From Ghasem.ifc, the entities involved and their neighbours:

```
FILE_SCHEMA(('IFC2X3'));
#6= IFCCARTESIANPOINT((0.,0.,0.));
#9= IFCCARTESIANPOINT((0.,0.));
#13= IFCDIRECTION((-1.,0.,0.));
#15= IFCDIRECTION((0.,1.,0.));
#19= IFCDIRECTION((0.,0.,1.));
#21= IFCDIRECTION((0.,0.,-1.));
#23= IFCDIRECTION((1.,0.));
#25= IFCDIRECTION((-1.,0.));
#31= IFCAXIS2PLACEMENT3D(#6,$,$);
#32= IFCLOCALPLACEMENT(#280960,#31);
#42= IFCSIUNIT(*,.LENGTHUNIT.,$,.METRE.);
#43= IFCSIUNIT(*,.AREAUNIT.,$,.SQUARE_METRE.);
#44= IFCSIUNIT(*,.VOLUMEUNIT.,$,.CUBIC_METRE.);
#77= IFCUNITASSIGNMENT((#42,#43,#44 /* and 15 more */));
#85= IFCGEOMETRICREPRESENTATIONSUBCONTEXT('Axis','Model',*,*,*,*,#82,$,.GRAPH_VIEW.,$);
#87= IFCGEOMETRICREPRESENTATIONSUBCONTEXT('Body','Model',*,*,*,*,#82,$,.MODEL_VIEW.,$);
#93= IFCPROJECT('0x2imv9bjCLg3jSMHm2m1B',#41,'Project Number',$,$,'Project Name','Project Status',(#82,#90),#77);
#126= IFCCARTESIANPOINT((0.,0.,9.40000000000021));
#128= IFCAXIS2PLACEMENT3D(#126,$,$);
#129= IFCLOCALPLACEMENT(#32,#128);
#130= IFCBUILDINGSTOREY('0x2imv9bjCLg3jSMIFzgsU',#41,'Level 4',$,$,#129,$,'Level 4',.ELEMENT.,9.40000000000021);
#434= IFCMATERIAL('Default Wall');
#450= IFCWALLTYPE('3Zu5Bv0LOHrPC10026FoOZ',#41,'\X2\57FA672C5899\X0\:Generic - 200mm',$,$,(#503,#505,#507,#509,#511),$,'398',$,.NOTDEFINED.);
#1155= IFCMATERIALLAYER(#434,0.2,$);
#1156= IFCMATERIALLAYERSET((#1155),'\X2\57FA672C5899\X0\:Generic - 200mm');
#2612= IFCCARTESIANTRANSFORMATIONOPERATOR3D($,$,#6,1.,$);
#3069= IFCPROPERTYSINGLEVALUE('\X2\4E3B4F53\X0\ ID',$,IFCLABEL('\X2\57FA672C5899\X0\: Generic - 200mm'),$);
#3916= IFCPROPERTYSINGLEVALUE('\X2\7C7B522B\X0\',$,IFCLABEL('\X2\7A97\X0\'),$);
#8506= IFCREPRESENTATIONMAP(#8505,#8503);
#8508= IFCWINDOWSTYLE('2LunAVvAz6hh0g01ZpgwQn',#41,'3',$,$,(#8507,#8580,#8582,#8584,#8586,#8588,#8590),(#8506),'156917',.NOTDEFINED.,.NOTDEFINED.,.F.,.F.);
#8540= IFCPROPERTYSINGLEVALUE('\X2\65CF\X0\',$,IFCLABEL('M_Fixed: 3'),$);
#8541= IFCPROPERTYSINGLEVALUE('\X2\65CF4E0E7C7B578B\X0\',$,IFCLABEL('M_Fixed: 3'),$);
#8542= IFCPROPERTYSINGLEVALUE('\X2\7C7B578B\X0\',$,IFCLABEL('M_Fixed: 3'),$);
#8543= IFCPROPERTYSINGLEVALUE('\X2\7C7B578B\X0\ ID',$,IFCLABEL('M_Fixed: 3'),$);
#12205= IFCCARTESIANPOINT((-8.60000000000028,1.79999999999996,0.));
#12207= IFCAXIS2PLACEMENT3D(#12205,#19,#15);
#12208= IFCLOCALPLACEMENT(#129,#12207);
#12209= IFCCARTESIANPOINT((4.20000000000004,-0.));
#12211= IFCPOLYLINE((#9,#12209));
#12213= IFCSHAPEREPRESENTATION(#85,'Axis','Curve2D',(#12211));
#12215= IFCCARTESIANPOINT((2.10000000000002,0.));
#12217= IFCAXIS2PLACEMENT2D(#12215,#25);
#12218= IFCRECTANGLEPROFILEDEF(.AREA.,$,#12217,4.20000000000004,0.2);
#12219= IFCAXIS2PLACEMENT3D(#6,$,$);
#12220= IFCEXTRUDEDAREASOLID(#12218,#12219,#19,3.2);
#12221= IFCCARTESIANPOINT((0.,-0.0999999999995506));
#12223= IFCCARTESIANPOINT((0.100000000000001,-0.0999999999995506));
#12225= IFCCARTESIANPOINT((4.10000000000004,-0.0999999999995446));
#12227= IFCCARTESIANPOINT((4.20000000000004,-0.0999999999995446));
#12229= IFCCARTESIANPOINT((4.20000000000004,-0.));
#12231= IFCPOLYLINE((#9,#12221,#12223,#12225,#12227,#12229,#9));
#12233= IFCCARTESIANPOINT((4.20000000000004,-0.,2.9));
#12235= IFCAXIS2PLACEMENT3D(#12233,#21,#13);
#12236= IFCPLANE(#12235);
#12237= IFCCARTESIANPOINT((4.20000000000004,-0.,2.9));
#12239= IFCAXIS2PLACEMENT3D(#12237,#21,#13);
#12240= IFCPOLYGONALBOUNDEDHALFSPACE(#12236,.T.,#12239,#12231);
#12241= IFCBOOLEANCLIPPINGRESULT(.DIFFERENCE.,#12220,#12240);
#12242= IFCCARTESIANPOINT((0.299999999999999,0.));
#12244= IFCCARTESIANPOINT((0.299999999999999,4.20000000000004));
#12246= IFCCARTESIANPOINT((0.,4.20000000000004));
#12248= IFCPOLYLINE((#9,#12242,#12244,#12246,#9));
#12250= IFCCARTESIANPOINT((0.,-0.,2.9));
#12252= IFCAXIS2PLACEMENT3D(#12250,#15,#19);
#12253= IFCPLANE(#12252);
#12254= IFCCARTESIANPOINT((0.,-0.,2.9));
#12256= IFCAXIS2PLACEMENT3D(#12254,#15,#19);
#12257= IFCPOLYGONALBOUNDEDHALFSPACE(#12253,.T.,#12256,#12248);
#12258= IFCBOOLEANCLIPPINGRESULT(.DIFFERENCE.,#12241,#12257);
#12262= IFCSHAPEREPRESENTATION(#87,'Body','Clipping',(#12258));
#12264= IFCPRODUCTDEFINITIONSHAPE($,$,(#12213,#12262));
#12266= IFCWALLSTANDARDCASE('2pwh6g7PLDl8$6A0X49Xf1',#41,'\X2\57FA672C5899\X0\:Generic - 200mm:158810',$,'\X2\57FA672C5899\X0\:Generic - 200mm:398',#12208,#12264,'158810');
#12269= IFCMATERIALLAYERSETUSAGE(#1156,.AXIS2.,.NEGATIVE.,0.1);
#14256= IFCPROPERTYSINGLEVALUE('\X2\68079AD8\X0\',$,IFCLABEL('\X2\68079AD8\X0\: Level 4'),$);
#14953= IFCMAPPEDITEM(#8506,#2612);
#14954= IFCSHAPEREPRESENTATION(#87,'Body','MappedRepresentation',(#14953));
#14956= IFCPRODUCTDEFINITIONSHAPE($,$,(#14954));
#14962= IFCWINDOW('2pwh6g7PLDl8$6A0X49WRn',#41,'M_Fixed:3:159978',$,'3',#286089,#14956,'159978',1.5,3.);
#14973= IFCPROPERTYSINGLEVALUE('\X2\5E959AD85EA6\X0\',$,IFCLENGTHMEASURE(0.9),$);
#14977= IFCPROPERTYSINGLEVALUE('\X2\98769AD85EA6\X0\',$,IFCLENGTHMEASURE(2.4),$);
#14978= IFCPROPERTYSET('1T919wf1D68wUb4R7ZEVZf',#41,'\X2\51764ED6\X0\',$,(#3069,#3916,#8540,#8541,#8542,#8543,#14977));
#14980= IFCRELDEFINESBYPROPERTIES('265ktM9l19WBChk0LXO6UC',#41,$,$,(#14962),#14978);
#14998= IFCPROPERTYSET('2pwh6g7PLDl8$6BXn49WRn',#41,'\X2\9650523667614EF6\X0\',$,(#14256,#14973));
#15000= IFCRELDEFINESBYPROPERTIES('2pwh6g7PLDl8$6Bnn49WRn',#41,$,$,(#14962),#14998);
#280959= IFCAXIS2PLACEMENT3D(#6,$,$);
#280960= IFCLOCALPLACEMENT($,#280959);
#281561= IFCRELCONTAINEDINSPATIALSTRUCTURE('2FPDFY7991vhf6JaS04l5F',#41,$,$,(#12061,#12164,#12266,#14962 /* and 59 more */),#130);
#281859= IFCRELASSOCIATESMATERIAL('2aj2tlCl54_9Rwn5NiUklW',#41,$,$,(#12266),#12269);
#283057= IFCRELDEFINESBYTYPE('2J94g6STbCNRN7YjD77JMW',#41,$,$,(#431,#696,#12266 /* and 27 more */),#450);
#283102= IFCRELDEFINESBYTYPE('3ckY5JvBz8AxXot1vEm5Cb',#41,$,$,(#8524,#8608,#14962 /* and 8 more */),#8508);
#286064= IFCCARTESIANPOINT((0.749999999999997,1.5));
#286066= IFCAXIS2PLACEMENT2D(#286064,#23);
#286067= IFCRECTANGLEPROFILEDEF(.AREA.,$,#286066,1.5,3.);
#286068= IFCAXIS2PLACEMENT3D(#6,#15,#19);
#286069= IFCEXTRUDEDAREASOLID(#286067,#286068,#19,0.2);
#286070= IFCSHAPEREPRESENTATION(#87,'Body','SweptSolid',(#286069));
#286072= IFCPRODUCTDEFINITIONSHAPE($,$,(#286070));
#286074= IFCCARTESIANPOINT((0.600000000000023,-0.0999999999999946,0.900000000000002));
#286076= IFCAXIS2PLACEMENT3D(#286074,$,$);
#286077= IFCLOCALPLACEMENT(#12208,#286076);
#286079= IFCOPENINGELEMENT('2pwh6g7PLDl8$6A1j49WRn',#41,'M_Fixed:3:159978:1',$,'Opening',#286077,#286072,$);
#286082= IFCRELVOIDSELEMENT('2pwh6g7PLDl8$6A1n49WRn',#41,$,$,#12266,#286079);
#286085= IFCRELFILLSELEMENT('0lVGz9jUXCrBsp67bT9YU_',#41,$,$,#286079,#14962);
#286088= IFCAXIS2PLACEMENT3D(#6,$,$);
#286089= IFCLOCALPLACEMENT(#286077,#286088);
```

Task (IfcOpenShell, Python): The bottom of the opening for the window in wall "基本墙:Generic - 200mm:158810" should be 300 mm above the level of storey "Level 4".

```python
import numpy as np
import ifcopenshell
import ifcopenshell.api.geometry
import ifcopenshell.api.pset
import ifcopenshell.geom
import ifcopenshell.util.element
import ifcopenshell.util.placement
import ifcopenshell.util.shape
import ifcopenshell.util.unit

model = ifcopenshell.open("Ghasem.ifc")
unit_scale = ifcopenshell.util.unit.calculate_unit_scale(model)

window = model.by_guid("2pwh6g7PLDl8$6A0X49WRn")
opening = window.FillsVoids[0].RelatingOpeningElement
storey = ifcopenshell.util.element.get_container(window, ifc_class="IfcBuildingStorey")
level = ifcopenshell.util.placement.get_local_placement(storey.ObjectPlacement)[2, 3]

# The opening's origin need not be at the sill, so measure its lowest point.
shape = ifcopenshell.geom.create_shape(ifcopenshell.geom.settings(), opening)
bottom = ifcopenshell.util.shape.get_shape_bottom_elevation(shape, shape.geometry) / unit_scale
dz = level + 0.3 - bottom

shift = np.array([0.0, 0.0, dz])
# The window is placed relative to its opening, so it follows when the opening moves.
matrix = ifcopenshell.util.placement.get_local_placement(opening.ObjectPlacement)
matrix[:3, 3] += shift
ifcopenshell.api.geometry.edit_object_placement(
    model, product=opening, matrix=matrix, is_si=False, should_transform_children=True
)

# Keep the stored heights in step.
pset = model.by_id(ifcopenshell.util.element.get_pset(window, "其他", should_inherit=False)["id"])
ifcopenshell.api.pset.edit_pset(model, pset=pset, properties={
    "顶高度": model.create_entity("IfcLengthMeasure", ifcopenshell.util.element.get_pset(window, "其他", "顶高度") + dz),
})
pset = model.by_id(ifcopenshell.util.element.get_pset(window, "限制条件", should_inherit=False)["id"])
ifcopenshell.api.pset.edit_pset(model, pset=pset, properties={
    "底高度": model.create_entity("IfcLengthMeasure", ifcopenshell.util.element.get_pset(window, "限制条件", "底高度") + dz),
})

print(f"moved by {dz * unit_scale:+.3f} m")

model.write("Ghasem-out.ifc")
```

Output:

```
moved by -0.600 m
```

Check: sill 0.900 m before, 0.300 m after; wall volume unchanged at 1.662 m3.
